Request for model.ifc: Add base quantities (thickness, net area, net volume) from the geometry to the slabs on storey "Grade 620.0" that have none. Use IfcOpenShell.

First a look at what the model holds.

```python
import ifcopenshell
import ifcopenshell.util.element
import ifcopenshell.util.unit

model = ifcopenshell.open("model.ifc")
print(model.schema)
for unit_type in ("LENGTHUNIT", "AREAUNIT", "VOLUMEUNIT"):
    print(unit_type, ifcopenshell.util.unit.calculate_unit_scale(model, unit_type))
storey = next(s for s in model.by_type("IfcBuildingStorey") if s.Name == "Grade 620.0")
slabs = [e for e in ifcopenshell.util.element.get_decomposition(storey) if e.is_a("IfcSlab")]
for e in sorted(slabs, key=lambda e: e.id()):
    print(e.id(), e.is_a(), e.Name, list(ifcopenshell.util.element.get_psets(e, qtos_only=True)), sep=" | ")
```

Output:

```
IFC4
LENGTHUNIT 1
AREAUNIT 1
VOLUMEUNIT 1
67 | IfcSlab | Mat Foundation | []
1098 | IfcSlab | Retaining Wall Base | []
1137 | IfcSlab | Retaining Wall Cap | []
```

```python
import ifcopenshell
import ifcopenshell.api.pset
import ifcopenshell.geom
import ifcopenshell.util.element
import ifcopenshell.util.shape
import ifcopenshell.util.unit

model = ifcopenshell.open("model.ifc")
unit_scale = ifcopenshell.util.unit.calculate_unit_scale(model)
area_scale = ifcopenshell.util.unit.calculate_unit_scale(model, "AREAUNIT")
volume_scale = ifcopenshell.util.unit.calculate_unit_scale(model, "VOLUMEUNIT")
settings = ifcopenshell.geom.settings()

storey = next(s for s in model.by_type("IfcBuildingStorey") if s.Name == "Grade 620.0")
slabs = [e for e in ifcopenshell.util.element.get_decomposition(storey) if e.is_a("IfcSlab")]

for e in sorted(slabs, key=lambda e: e.id()):
    if ifcopenshell.util.element.get_psets(e, qtos_only=True, should_inherit=False):
        continue
    # Geometry comes back in metres, in the element's own axes.
    shape = ifcopenshell.geom.create_shape(settings, e)
    values = {
        "Width": ifcopenshell.util.shape.get_z(shape.geometry) / unit_scale,
        "NetArea": ifcopenshell.util.shape.get_footprint_area(shape.geometry) / area_scale,
        "NetVolume": ifcopenshell.util.shape.get_volume(shape.geometry) / volume_scale,
    }
    qto = ifcopenshell.api.pset.add_qto(model, product=e, name="Qto_SlabBaseQuantities")
    ifcopenshell.api.pset.edit_qto(model, qto=qto, properties=values)
    print(e.id(), {k: round(v, 3) for k, v in values.items()})

model.write("model_rev.ifc")
```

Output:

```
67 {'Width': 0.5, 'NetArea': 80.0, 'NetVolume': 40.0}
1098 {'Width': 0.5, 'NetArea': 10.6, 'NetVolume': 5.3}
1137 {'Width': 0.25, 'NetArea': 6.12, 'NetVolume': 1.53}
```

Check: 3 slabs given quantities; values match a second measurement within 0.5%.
